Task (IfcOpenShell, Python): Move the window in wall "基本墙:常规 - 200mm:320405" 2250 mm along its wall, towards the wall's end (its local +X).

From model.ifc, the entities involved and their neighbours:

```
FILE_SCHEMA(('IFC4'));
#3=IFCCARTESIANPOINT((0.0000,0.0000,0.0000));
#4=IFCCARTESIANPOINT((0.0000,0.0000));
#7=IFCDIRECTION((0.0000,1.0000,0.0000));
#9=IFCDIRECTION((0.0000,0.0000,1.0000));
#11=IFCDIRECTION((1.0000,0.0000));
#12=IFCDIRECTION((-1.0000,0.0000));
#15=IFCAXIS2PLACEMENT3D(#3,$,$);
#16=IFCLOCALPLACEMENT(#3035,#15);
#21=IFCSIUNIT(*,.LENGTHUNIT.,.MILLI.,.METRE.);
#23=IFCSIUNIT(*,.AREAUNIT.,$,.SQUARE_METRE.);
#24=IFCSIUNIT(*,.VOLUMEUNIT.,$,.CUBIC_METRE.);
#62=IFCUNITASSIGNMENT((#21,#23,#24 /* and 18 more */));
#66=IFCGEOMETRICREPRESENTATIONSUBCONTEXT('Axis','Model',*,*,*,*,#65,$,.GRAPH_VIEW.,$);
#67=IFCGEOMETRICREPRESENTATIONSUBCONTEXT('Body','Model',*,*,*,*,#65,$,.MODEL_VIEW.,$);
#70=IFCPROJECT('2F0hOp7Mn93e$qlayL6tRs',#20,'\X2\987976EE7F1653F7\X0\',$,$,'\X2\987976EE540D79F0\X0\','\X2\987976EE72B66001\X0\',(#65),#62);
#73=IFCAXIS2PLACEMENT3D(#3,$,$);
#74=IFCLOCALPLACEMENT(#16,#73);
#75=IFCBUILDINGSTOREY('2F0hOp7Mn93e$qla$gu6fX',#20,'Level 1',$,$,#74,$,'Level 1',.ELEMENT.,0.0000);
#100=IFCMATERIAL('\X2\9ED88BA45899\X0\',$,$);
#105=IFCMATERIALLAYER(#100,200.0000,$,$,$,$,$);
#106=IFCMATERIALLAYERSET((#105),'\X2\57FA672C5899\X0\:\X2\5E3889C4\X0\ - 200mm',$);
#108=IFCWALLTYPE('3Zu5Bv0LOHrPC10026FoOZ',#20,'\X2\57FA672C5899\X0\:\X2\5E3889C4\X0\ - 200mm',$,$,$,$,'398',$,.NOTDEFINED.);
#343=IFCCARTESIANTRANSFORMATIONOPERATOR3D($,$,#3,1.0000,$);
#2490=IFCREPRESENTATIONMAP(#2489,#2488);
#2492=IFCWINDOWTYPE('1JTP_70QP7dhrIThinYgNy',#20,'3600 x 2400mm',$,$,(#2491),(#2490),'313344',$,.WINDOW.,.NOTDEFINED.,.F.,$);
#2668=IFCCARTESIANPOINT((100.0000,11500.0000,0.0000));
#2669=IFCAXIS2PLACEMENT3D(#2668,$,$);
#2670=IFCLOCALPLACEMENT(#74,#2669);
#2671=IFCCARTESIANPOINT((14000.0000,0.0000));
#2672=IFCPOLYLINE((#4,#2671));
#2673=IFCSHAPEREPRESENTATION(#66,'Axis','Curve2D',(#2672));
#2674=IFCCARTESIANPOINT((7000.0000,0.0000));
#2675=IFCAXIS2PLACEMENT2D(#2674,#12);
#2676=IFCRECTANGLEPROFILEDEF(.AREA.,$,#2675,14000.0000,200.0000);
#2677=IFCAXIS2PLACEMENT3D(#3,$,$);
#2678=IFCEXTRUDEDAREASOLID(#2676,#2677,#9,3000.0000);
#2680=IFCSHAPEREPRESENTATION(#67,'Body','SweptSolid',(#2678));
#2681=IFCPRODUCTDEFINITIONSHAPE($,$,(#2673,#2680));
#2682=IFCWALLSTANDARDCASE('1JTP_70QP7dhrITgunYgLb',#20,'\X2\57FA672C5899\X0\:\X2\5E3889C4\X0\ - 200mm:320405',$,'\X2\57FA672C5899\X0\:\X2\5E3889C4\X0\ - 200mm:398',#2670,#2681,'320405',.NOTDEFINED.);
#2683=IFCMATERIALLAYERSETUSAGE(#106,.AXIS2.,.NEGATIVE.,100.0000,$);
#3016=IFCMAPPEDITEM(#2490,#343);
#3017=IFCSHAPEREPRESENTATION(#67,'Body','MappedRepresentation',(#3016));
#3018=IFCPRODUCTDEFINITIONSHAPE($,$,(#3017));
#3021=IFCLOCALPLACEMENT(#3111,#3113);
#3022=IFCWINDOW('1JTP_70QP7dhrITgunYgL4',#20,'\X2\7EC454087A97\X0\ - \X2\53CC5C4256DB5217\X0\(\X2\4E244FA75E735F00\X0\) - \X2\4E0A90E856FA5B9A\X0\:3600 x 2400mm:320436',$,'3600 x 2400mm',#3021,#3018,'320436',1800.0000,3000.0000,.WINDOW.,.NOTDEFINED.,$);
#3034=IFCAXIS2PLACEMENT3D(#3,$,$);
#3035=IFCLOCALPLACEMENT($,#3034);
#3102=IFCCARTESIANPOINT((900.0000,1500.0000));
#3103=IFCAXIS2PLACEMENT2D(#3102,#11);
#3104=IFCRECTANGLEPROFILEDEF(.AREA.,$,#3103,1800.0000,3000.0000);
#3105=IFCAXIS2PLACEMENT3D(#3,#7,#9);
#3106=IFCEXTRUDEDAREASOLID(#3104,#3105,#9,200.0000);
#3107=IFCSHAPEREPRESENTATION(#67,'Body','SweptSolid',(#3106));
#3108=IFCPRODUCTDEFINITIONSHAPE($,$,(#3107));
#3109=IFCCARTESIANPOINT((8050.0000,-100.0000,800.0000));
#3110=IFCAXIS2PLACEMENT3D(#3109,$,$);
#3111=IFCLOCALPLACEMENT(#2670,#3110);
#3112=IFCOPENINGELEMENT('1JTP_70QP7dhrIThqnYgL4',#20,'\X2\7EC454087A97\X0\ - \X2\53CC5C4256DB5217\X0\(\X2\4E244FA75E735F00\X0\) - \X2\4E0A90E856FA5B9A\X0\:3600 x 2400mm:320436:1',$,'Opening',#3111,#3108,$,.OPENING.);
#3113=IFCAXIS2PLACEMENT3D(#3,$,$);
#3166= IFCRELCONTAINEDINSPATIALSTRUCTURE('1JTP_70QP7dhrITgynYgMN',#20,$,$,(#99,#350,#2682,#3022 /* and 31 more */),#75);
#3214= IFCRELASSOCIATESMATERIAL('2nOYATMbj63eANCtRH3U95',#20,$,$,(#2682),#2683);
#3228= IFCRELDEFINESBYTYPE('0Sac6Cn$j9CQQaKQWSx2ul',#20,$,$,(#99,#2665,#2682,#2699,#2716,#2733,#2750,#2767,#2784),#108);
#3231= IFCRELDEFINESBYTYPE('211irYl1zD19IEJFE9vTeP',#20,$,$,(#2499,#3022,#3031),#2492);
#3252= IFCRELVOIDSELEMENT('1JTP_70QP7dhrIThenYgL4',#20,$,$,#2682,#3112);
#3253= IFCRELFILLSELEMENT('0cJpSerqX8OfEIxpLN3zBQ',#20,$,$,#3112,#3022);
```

```python
import ifcopenshell
import ifcopenshell.api.geometry
import ifcopenshell.util.placement
import ifcopenshell.util.unit

model = ifcopenshell.open("model.ifc")
unit_scale = ifcopenshell.util.unit.calculate_unit_scale(model)

window = model.by_guid("1JTP_70QP7dhrITgunYgL4")
opening = window.FillsVoids[0].RelatingOpeningElement
wall = opening.VoidsElements[0].RelatingBuildingElement

wall_matrix = ifcopenshell.util.placement.get_local_placement(wall.ObjectPlacement)
shift = wall_matrix[:3, 0] * 2.25 / unit_scale
before = ifcopenshell.util.placement.get_local_placement(window.ObjectPlacement)[:3, 3].copy()

# The window is placed relative to its opening, so it follows when the opening moves.
matrix = ifcopenshell.util.placement.get_local_placement(opening.ObjectPlacement)
matrix[:3, 3] += shift
ifcopenshell.api.geometry.edit_object_placement(
    model, product=opening, matrix=matrix, is_si=False, should_transform_children=True
)

after = ifcopenshell.util.placement.get_local_placement(window.ObjectPlacement)[:3, 3]
print("window moved by", (after - before).round(3) + 0.0)

model.write("model_updated.ifc")
```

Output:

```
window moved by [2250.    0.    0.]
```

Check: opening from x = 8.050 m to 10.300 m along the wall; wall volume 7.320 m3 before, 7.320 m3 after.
